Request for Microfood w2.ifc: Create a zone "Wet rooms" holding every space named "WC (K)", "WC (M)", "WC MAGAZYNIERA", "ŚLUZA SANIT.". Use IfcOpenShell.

First a look at what the model holds.

```python
import ifcopenshell

model = ifcopenshell.open("Microfood w2.ifc")
print(model.schema)
seen = {}
for space in model.by_type("IfcSpace"):
    seen[space.LongName] = seen.get(space.LongName, 0) + 1
for name, count in sorted(seen.items(), key=str):
    print(count, "x", name)
print("zones:", [z.Name for z in model.by_type("IfcZone")][:20])
```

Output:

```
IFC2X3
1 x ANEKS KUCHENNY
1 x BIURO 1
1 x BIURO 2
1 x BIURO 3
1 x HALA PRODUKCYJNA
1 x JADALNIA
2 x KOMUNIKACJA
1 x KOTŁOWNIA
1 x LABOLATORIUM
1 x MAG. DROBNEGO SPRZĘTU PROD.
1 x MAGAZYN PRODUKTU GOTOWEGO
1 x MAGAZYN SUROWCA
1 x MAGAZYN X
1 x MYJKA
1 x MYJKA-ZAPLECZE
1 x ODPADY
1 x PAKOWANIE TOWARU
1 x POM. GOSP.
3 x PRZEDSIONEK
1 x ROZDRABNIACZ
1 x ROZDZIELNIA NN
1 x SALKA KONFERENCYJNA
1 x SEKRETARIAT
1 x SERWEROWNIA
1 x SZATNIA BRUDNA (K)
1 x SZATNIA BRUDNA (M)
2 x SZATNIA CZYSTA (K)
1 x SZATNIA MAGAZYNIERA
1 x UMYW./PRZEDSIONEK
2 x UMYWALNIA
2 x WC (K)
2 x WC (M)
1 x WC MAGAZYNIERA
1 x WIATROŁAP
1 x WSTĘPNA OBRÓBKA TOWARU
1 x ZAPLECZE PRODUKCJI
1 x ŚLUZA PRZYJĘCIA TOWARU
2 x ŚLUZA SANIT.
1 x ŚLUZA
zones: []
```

```python
import ifcopenshell
import ifcopenshell.api.group
import ifcopenshell.api.root

model = ifcopenshell.open("Microfood w2.ifc")

names = {"WC (K)", "WC (M)", "WC MAGAZYNIERA", "ŚLUZA SANIT."}
spaces = [s for s in model.by_type("IfcSpace") if s.LongName in names]

zone = ifcopenshell.api.root.create_entity(model, ifc_class="IfcZone", name="Wet rooms")
ifcopenshell.api.group.assign_group(model, products=spaces, group=zone)
print(len(spaces), "spaces in", zone.Name)

model.write("Microfood w2_v2.ifc")
```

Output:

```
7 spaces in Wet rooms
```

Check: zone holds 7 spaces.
